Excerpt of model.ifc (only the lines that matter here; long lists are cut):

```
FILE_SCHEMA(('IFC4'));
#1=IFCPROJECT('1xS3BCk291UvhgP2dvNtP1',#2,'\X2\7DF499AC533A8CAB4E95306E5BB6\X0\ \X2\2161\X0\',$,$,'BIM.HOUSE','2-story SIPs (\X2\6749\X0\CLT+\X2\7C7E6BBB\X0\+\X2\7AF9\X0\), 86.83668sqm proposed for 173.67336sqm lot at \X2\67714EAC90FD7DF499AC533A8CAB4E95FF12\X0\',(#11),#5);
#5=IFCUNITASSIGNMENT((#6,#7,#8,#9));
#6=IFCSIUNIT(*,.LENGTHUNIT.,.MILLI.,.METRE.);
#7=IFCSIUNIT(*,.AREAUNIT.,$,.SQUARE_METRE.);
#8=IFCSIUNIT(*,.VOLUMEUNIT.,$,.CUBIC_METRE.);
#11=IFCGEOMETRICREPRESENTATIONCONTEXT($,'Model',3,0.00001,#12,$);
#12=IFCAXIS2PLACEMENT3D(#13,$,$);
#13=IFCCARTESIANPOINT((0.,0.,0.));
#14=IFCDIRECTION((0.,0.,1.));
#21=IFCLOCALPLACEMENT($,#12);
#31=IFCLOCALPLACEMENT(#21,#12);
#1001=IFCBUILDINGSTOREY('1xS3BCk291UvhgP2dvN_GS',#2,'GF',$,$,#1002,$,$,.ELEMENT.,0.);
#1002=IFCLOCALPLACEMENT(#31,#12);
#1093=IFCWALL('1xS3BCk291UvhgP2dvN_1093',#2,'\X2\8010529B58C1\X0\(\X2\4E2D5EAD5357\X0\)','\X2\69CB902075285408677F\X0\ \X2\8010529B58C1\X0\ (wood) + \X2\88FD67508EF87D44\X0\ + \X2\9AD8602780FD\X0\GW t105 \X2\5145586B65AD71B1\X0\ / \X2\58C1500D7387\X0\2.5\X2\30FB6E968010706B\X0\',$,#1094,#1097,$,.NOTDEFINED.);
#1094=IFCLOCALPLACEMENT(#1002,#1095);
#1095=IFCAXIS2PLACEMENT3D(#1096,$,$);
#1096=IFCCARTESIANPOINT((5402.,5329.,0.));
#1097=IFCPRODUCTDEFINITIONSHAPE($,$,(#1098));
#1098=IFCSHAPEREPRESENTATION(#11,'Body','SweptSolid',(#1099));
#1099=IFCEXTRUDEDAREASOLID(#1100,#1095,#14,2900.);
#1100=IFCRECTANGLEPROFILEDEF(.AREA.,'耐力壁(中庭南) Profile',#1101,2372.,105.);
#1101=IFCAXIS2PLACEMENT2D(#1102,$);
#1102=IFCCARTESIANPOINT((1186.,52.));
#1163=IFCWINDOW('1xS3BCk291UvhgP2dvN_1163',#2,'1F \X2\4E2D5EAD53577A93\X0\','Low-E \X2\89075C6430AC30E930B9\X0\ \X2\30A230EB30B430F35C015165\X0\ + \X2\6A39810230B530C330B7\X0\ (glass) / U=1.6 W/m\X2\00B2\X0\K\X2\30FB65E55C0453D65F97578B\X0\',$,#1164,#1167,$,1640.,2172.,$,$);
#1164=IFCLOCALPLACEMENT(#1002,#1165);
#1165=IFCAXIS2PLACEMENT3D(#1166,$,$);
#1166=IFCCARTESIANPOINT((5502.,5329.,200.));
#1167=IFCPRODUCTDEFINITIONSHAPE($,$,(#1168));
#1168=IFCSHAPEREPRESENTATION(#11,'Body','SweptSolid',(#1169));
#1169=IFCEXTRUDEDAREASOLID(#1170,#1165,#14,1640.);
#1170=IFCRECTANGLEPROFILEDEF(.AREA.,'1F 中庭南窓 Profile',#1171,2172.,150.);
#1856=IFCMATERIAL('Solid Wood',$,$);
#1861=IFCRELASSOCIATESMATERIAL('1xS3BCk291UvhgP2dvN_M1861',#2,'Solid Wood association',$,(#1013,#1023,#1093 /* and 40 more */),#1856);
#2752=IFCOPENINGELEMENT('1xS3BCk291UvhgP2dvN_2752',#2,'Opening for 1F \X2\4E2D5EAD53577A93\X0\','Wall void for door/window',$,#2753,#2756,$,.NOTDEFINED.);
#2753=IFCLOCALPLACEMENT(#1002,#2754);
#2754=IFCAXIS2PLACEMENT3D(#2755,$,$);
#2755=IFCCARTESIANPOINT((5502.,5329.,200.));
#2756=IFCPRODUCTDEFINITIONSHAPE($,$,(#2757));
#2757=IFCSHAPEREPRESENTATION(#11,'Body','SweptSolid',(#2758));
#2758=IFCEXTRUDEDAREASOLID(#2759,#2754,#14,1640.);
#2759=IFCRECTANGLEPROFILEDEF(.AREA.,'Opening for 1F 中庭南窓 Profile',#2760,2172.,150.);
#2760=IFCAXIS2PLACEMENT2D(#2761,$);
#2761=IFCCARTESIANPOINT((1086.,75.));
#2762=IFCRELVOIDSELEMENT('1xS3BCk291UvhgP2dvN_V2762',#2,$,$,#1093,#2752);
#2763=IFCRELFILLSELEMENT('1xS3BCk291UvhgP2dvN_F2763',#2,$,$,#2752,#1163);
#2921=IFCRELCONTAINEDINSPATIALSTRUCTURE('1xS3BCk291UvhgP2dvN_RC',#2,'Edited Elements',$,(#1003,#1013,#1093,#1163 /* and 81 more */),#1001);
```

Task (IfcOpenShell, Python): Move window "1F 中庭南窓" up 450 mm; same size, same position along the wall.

```python
import numpy as np
import ifcopenshell
import ifcopenshell.api.geometry
import ifcopenshell.util.placement
import ifcopenshell.util.unit

model = ifcopenshell.open("model.ifc")
unit_scale = ifcopenshell.util.unit.calculate_unit_scale(model)

window = model.by_id(1163)
opening = window.FillsVoids[0].RelatingOpeningElement
dz = 0.45 / unit_scale

shift = np.array([0.0, 0.0, dz])
# The window is not placed relative to its opening, so move both.
for product in (opening, window):
    matrix = ifcopenshell.util.placement.get_local_placement(product.ObjectPlacement)
    matrix[:3, 3] += shift
    ifcopenshell.api.geometry.edit_object_placement(model, product=product, matrix=matrix, is_si=False)

print(f"moved by {dz * unit_scale:+.3f} m")

model.write("model_edited.ifc")
```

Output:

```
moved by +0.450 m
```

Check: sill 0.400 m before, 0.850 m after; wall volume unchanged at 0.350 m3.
